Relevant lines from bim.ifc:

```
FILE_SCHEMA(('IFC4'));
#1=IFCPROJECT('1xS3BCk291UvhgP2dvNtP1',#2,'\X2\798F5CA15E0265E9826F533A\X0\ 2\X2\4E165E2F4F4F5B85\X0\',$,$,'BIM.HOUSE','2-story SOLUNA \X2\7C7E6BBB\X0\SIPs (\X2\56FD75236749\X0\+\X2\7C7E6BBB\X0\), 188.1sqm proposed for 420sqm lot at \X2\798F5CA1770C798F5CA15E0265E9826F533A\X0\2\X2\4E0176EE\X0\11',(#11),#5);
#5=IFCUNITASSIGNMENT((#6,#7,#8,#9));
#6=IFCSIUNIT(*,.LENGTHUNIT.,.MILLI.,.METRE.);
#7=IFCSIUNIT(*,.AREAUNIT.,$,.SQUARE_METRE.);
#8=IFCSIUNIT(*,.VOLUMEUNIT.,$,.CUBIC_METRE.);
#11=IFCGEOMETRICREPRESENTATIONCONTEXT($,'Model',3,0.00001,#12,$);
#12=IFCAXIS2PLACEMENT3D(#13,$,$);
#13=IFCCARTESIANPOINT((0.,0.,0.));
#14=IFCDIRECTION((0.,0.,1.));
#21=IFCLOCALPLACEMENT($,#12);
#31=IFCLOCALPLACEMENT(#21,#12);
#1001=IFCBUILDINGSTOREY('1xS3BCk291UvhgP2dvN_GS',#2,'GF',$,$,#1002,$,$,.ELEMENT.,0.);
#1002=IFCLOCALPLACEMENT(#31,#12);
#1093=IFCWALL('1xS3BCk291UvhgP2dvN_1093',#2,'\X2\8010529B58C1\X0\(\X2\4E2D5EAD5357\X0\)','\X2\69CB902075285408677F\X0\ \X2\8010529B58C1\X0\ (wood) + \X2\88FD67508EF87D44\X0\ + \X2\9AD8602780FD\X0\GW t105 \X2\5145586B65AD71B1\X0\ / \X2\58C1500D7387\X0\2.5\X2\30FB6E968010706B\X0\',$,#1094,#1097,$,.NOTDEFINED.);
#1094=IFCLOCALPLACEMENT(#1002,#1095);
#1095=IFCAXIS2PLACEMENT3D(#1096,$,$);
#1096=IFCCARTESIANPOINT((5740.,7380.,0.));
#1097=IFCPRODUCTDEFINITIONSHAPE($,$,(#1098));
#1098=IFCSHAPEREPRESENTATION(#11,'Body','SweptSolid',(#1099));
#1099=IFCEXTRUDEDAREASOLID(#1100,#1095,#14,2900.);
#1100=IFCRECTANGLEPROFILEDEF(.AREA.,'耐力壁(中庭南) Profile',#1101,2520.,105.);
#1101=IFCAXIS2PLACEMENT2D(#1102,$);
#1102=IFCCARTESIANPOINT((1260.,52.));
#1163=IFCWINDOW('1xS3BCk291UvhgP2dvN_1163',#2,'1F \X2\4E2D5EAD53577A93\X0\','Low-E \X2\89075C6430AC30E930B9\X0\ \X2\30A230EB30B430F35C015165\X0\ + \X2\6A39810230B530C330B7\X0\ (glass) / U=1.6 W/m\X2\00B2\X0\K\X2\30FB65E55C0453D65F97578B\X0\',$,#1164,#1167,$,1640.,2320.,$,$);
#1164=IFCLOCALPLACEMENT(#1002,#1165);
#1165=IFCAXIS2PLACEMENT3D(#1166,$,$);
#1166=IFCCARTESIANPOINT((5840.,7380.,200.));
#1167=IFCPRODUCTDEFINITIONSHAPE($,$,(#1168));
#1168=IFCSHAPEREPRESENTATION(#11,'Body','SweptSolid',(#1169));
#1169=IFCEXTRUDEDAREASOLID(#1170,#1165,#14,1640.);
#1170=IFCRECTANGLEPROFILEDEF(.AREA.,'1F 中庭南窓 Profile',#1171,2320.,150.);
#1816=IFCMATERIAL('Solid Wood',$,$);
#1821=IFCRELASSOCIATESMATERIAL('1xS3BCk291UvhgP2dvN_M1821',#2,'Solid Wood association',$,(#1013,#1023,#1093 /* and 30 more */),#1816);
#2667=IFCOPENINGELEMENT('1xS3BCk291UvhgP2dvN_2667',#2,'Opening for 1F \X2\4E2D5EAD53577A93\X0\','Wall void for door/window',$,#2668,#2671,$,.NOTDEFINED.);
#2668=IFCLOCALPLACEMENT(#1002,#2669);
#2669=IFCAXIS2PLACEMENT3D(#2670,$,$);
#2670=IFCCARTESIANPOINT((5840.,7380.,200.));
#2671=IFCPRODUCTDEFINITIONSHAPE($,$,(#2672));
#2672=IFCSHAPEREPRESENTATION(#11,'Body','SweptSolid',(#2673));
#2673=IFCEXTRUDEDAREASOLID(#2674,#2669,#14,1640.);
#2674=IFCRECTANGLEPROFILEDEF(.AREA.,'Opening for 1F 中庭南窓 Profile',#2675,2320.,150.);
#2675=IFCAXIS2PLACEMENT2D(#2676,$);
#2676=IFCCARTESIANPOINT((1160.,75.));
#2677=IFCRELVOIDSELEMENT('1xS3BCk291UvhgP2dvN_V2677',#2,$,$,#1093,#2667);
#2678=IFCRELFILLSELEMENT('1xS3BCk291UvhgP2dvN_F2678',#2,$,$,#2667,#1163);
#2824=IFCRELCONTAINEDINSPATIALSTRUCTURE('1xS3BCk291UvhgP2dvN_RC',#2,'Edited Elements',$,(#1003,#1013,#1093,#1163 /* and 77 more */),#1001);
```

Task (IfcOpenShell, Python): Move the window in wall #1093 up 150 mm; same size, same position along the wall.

```python
import numpy as np
import ifcopenshell
import ifcopenshell.api.geometry
import ifcopenshell.util.placement
import ifcopenshell.util.unit

model = ifcopenshell.open("bim.ifc")
unit_scale = ifcopenshell.util.unit.calculate_unit_scale(model)

window = model.by_guid("1xS3BCk291UvhgP2dvN_1163")
opening = window.FillsVoids[0].RelatingOpeningElement
dz = 150.0

shift = np.array([0.0, 0.0, dz])
# The window is not placed relative to its opening, so move both.
for product in (opening, window):
    matrix = ifcopenshell.util.placement.get_local_placement(product.ObjectPlacement)
    matrix[:3, 3] += shift
    ifcopenshell.api.geometry.edit_object_placement(model, product=product, matrix=matrix, is_si=False)

print(f"moved by {dz * unit_scale:+.3f} m")

model.write("bim-out.ifc")
```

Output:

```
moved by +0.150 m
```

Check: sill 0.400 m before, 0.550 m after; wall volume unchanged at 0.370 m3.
